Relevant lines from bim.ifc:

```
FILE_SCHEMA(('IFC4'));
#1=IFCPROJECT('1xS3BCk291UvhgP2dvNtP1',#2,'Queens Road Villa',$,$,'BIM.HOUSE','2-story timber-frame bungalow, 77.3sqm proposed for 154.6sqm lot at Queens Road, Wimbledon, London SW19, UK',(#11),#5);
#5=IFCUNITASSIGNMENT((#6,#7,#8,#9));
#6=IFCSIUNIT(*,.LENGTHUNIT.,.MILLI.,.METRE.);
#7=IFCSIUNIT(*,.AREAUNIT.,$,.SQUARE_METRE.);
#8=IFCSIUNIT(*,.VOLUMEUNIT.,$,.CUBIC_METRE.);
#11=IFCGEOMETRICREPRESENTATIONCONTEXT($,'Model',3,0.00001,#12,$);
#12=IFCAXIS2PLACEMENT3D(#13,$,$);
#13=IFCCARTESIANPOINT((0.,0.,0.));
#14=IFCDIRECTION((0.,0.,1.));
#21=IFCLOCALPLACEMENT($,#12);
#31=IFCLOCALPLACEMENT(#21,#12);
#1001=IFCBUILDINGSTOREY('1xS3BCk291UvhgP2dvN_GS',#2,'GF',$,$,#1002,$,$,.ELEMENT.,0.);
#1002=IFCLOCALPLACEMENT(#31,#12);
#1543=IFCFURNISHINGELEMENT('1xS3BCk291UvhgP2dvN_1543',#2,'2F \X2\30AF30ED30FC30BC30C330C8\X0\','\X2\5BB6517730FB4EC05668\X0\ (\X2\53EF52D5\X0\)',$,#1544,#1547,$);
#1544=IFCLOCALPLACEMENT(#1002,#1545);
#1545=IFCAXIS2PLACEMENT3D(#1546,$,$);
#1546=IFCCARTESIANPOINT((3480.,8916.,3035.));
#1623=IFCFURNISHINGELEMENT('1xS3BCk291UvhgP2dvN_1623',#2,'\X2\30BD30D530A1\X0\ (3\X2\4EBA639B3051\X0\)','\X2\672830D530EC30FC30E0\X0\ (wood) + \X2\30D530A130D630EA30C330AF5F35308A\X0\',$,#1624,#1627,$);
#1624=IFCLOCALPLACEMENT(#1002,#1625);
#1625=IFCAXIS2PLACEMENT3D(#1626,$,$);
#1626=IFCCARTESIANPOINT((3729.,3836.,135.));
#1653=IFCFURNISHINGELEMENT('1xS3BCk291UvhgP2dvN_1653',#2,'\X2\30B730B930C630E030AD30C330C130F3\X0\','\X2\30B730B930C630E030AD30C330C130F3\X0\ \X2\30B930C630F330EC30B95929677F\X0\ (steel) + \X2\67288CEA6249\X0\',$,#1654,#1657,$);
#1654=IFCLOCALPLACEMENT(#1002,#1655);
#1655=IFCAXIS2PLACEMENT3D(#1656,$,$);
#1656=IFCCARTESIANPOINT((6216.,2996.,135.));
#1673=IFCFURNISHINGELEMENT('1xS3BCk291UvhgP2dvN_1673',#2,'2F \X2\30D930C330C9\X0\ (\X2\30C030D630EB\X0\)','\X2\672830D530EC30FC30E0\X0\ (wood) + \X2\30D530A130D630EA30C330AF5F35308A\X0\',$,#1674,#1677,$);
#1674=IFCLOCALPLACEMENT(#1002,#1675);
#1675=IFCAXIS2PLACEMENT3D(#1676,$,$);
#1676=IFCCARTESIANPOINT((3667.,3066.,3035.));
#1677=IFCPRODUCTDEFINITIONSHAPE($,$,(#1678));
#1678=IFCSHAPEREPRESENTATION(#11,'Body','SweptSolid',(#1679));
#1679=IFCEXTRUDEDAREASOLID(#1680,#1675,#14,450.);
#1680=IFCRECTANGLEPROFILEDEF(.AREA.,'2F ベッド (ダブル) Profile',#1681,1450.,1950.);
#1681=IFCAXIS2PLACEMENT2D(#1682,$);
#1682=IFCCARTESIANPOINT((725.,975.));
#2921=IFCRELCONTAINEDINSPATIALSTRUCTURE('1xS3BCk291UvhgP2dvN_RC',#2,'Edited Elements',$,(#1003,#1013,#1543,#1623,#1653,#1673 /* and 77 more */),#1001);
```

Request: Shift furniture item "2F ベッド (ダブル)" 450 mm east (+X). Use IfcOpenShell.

```python
import ifcopenshell
import ifcopenshell.api.geometry
import ifcopenshell.util.placement
import ifcopenshell.util.unit

model = ifcopenshell.open("bim.ifc")
unit_scale = ifcopenshell.util.unit.calculate_unit_scale(model)

item = model.by_guid("1xS3BCk291UvhgP2dvN_1673")
matrix = ifcopenshell.util.placement.get_local_placement(item.ObjectPlacement)
matrix[0, 3] += 0.45 / unit_scale
ifcopenshell.api.geometry.edit_object_placement(model, product=item, matrix=matrix, is_si=False)

print(ifcopenshell.util.placement.get_local_placement(item.ObjectPlacement).round(3) + 0.0)

model.write("bim-out.ifc")
```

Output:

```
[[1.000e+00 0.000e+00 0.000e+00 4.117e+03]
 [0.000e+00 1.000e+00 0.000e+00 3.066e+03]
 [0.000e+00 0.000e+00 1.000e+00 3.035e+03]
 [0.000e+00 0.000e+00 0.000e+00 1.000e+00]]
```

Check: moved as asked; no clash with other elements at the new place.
